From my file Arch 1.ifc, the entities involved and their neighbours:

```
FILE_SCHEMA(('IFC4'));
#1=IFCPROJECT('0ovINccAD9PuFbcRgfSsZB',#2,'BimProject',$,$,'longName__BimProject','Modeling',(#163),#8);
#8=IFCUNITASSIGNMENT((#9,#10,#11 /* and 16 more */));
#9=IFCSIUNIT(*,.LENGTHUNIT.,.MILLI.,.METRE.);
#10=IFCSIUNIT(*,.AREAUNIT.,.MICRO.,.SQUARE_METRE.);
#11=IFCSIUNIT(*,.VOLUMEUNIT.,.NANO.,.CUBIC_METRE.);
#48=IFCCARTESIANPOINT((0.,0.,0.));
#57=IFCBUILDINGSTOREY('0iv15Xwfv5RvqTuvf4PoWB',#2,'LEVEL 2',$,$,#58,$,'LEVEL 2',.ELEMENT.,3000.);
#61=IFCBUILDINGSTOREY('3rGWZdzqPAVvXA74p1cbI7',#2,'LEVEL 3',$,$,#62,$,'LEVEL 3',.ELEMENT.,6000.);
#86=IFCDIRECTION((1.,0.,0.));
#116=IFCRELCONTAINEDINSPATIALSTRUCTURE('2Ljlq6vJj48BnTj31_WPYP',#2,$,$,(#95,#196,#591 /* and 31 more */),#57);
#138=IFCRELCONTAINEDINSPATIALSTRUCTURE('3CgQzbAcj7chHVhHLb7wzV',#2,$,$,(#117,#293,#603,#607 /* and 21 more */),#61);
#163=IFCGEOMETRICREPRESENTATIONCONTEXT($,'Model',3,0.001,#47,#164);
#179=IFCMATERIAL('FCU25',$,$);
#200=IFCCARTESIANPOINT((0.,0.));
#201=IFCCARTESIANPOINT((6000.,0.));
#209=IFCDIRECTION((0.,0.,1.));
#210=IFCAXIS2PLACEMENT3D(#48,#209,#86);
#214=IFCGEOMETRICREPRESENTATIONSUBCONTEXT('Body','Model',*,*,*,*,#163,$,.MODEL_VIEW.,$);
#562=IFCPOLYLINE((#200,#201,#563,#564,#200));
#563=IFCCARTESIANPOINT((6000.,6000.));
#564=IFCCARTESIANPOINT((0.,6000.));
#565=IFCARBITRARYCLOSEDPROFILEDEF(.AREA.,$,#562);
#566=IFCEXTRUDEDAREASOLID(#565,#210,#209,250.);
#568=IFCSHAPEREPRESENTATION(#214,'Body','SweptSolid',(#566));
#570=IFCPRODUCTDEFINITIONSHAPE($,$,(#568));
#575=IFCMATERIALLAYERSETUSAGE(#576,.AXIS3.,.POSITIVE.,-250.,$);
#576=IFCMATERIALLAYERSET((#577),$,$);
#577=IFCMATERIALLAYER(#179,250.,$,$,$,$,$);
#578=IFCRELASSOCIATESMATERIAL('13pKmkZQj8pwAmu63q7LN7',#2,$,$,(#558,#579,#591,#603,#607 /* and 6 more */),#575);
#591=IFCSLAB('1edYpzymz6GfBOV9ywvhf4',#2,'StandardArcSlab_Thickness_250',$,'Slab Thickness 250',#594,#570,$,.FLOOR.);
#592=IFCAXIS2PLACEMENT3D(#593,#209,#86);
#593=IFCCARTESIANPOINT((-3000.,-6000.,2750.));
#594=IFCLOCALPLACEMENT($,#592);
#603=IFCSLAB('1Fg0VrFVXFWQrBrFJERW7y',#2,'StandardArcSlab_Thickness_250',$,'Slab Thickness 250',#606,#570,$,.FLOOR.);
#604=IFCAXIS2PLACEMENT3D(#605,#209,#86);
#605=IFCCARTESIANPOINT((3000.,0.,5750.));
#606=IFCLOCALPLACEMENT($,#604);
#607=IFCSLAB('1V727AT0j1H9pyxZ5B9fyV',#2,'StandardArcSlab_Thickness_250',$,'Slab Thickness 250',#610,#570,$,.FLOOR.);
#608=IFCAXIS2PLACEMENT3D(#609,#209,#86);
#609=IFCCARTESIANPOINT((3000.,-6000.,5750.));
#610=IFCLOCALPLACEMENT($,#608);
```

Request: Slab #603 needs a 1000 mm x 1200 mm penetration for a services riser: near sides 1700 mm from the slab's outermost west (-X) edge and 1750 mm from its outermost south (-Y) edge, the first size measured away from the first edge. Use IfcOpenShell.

```python
import numpy as np
import ifcopenshell
import ifcopenshell.api.feature
import ifcopenshell.api.geometry
import ifcopenshell.api.root
import ifcopenshell.geom
import ifcopenshell.util.placement
import ifcopenshell.util.representation
import ifcopenshell.util.shape
import ifcopenshell.util.unit

model = ifcopenshell.open("my file Arch 1.ifc")
unit_scale = ifcopenshell.util.unit.calculate_unit_scale(model)
settings = ifcopenshell.geom.settings()


def volume(element):
    """Net volume in cubic metres, openings subtracted."""
    shape = ifcopenshell.geom.create_shape(settings, element)
    return ifcopenshell.util.shape.get_volume(shape.geometry)


slab = model.by_id(603)
before = volume(slab)

# Extent in the slab's own axes, in metres. The edges named are its -X and -Y sides.
slab_shape = ifcopenshell.geom.create_shape(settings, slab)
vertices = ifcopenshell.util.shape.get_vertices(slab_shape.geometry)
x_min, y_min, bottom = vertices.min(axis=0)
top = vertices[:, 2].max()

opening = ifcopenshell.api.root.create_entity(model, ifc_class="IfcOpeningElement", name="Services riser opening", predefined_type="OPENING")
context = ifcopenshell.util.representation.get_context(model, "Model", "Body", "MODEL_VIEW")
width, depth = 1, 1.2
outline = [(0.0, 0.0), (width, 0.0), (width, depth), (0.0, depth), (0.0, 0.0)]
# Overshoot both faces by 50 mm so the cut is clean.
shape = ifcopenshell.api.geometry.add_slab_representation(
    model, context=context, depth=top - bottom + 0.1, polyline=outline
)
ifcopenshell.api.geometry.assign_representation(model, product=opening, representation=shape)

matrix = ifcopenshell.util.placement.get_local_placement(slab.ObjectPlacement)
matrix[:, 3] = matrix @ np.append(np.array([x_min + 1.7, y_min + 1.75, bottom - 0.05]) / unit_scale, 1.0)
ifcopenshell.api.geometry.edit_object_placement(model, product=opening, matrix=matrix, is_si=False)
ifcopenshell.api.feature.add_feature(model, feature=opening, element=slab)

after = volume(slab)

print(f"slab volume {before:.3f} -> {after:.3f} m3")

model.write("my file Arch 1_updated.ifc")
```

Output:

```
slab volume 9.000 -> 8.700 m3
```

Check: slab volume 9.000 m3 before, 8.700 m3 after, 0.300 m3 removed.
